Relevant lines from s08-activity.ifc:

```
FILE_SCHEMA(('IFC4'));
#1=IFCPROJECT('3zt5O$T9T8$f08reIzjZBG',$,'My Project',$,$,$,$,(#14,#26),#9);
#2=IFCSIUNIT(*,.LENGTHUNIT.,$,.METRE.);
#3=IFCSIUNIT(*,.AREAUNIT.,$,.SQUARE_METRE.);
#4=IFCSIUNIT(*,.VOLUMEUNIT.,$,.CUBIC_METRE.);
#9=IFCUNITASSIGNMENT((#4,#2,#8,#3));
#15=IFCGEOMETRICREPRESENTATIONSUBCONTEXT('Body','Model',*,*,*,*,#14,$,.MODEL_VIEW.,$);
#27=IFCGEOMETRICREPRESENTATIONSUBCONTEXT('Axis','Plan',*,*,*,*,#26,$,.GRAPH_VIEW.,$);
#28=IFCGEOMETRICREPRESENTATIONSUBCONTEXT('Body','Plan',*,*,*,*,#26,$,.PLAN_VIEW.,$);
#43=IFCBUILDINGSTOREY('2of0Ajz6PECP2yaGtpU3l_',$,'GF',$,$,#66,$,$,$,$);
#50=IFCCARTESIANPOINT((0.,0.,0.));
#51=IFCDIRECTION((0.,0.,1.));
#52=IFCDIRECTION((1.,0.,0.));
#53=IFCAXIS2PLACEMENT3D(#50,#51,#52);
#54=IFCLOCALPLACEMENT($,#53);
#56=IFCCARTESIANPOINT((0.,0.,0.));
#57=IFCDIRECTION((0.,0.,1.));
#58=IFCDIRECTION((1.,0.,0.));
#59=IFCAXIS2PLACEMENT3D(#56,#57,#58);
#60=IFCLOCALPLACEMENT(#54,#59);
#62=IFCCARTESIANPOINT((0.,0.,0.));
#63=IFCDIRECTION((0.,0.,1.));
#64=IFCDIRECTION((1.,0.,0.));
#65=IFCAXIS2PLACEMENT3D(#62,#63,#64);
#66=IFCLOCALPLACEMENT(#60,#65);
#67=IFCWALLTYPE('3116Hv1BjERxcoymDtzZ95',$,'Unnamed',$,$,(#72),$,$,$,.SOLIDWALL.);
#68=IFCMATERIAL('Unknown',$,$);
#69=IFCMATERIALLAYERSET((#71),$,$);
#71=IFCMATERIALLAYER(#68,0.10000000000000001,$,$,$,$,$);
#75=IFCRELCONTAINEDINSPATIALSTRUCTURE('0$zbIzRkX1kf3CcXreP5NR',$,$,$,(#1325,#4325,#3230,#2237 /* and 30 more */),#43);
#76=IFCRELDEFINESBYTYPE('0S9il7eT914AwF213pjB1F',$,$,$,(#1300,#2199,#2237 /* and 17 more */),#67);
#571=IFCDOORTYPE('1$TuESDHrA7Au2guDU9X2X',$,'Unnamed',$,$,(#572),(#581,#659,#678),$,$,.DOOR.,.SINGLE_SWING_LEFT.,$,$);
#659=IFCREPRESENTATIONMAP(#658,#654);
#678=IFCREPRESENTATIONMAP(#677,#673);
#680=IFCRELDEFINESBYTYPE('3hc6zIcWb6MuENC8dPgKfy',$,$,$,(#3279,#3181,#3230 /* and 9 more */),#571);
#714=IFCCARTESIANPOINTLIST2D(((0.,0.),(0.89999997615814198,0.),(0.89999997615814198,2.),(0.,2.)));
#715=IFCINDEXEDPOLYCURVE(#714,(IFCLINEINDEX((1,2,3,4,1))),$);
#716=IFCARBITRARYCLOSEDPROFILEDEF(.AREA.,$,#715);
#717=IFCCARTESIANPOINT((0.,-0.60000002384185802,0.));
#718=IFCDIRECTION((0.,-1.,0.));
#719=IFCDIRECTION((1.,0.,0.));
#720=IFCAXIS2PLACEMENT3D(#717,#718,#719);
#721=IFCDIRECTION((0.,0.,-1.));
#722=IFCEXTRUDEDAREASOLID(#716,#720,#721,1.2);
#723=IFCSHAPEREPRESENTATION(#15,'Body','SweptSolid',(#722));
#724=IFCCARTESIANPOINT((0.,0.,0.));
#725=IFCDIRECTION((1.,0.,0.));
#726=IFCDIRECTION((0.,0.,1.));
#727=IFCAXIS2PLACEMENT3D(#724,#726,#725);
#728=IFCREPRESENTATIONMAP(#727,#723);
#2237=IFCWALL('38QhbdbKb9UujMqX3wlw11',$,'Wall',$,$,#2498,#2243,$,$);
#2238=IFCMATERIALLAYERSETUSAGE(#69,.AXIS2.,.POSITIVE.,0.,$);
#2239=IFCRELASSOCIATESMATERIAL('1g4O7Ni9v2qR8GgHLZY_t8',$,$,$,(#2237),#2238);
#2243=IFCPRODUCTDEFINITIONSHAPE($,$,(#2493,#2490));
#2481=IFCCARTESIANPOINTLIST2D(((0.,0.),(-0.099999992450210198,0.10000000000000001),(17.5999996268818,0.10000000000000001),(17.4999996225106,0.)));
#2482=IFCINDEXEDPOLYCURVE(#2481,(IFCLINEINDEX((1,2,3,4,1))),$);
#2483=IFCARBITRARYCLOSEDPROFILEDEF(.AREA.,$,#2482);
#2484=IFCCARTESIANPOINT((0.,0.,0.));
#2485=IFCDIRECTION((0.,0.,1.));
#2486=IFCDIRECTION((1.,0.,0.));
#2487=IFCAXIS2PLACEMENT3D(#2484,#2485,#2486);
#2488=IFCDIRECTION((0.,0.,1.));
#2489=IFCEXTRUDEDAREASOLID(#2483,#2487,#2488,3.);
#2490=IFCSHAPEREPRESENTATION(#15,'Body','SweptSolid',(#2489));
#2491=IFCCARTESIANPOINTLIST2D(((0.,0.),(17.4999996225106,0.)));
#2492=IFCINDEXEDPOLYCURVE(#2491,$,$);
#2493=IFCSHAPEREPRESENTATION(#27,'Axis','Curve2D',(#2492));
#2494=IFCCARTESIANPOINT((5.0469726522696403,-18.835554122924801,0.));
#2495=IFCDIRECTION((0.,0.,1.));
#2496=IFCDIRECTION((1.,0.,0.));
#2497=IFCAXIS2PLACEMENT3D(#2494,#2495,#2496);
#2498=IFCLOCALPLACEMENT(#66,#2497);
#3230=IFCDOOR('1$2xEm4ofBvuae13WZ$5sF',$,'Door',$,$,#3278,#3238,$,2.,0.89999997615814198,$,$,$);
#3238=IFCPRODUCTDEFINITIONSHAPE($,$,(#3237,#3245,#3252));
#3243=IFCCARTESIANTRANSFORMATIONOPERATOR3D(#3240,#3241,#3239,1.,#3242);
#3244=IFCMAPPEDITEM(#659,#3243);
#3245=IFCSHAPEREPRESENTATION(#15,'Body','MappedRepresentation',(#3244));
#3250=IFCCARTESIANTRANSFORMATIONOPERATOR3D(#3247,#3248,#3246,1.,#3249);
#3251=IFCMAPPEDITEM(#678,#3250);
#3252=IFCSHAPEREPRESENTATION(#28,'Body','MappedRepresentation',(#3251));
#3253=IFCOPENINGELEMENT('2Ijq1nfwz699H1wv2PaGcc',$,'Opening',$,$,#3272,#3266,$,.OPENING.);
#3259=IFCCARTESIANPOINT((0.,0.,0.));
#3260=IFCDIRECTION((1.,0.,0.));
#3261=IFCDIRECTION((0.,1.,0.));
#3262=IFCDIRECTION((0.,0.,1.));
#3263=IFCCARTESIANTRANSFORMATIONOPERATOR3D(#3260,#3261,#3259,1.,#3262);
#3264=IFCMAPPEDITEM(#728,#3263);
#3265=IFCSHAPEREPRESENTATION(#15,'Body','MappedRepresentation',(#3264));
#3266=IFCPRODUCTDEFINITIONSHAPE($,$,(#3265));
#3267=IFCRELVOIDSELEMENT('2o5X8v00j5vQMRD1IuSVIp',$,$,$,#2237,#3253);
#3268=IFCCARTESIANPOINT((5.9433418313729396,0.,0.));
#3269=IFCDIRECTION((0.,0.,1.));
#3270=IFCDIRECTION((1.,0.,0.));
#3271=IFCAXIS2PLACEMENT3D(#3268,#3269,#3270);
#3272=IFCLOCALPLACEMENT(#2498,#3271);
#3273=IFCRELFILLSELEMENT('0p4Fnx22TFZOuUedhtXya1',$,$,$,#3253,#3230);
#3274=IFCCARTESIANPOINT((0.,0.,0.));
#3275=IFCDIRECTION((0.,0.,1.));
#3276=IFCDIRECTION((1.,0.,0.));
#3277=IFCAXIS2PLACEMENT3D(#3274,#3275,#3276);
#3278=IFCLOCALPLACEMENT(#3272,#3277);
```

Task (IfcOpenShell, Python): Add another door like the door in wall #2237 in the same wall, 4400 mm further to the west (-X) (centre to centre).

```python
import ifcopenshell
import ifcopenshell.api.feature
import ifcopenshell.api.geometry
import ifcopenshell.api.root
import ifcopenshell.geom
import ifcopenshell.util.element
import ifcopenshell.util.placement
import ifcopenshell.util.shape
import ifcopenshell.util.unit

model = ifcopenshell.open("s08-activity.ifc")
unit_scale = ifcopenshell.util.unit.calculate_unit_scale(model)
settings = ifcopenshell.geom.settings()


def volume(element):
    """Net volume in cubic metres, openings subtracted."""
    shape = ifcopenshell.geom.create_shape(settings, element)
    return ifcopenshell.util.shape.get_volume(shape.geometry)


door = model.by_guid("1$2xEm4ofBvuae13WZ$5sF")
opening = door.FillsVoids[0].RelatingOpeningElement
wall = opening.VoidsElements[0].RelatingBuildingElement
before = volume(wall)
shift = ifcopenshell.util.placement.get_local_placement(wall.ObjectPlacement)[:3, 0] * -4.4 / unit_scale

# copy_class copies the void relationship, type, container and properties, but no geometry.
new_opening = ifcopenshell.api.root.copy_class(model, product=opening)
new_opening.Representation = ifcopenshell.util.element.copy_deep(
    model, opening.Representation, exclude=["IfcGeometricRepresentationContext", "IfcRepresentationMap"]
)
new_door = ifcopenshell.api.root.copy_class(model, product=door)
new_door.Representation = ifcopenshell.util.element.copy_deep(
    model, door.Representation, exclude=["IfcGeometricRepresentationContext", "IfcRepresentationMap"]
)
ifcopenshell.api.feature.add_filling(model, opening=new_opening, element=new_door)

for old, new in ((opening, new_opening), (door, new_door)):
    matrix = ifcopenshell.util.placement.get_local_placement(old.ObjectPlacement)
    matrix[:3, 3] += shift
    ifcopenshell.api.geometry.edit_object_placement(model, product=new, matrix=matrix, is_si=False)

after = volume(wall)

print(f"wall volume {before:.3f} -> {after:.3f} m3")

model.write("s08-activity-out.ifc")
```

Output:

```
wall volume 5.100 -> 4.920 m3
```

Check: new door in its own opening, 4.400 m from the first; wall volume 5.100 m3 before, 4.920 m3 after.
